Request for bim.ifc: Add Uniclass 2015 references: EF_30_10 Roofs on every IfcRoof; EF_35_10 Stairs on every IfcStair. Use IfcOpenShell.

First a look at what the model holds.

```python
import ifcopenshell

model = ifcopenshell.open("bim.ifc")
print(model.schema)
print("classifications:", [c.Name for c in model.by_type("IfcClassification")])
for ifc_class in ("IfcDoor", "IfcRoof", "IfcStair", "IfcWall", "IfcWindow"):
    print(ifc_class, len(model.by_type(ifc_class)))
```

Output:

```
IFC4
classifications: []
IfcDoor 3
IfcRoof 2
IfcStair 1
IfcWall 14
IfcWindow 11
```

```python
import ifcopenshell
import ifcopenshell.api.classification

model = ifcopenshell.open("bim.ifc")

system = ifcopenshell.api.classification.add_classification(model, classification="Uniclass 2015")

codes = {
    "IfcRoof": ("EF_30_10", "Roofs"),
    "IfcStair": ("EF_35_10", "Stairs"),
}
for ifc_class, (code, name) in codes.items():
    products = model.by_type(ifc_class)
    ifcopenshell.api.classification.add_reference(
        model, products=products, classification=system, identification=code, name=name
    )
    print(code, len(products))

model.write("bim_updated.ifc")
```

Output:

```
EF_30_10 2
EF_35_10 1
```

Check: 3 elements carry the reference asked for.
